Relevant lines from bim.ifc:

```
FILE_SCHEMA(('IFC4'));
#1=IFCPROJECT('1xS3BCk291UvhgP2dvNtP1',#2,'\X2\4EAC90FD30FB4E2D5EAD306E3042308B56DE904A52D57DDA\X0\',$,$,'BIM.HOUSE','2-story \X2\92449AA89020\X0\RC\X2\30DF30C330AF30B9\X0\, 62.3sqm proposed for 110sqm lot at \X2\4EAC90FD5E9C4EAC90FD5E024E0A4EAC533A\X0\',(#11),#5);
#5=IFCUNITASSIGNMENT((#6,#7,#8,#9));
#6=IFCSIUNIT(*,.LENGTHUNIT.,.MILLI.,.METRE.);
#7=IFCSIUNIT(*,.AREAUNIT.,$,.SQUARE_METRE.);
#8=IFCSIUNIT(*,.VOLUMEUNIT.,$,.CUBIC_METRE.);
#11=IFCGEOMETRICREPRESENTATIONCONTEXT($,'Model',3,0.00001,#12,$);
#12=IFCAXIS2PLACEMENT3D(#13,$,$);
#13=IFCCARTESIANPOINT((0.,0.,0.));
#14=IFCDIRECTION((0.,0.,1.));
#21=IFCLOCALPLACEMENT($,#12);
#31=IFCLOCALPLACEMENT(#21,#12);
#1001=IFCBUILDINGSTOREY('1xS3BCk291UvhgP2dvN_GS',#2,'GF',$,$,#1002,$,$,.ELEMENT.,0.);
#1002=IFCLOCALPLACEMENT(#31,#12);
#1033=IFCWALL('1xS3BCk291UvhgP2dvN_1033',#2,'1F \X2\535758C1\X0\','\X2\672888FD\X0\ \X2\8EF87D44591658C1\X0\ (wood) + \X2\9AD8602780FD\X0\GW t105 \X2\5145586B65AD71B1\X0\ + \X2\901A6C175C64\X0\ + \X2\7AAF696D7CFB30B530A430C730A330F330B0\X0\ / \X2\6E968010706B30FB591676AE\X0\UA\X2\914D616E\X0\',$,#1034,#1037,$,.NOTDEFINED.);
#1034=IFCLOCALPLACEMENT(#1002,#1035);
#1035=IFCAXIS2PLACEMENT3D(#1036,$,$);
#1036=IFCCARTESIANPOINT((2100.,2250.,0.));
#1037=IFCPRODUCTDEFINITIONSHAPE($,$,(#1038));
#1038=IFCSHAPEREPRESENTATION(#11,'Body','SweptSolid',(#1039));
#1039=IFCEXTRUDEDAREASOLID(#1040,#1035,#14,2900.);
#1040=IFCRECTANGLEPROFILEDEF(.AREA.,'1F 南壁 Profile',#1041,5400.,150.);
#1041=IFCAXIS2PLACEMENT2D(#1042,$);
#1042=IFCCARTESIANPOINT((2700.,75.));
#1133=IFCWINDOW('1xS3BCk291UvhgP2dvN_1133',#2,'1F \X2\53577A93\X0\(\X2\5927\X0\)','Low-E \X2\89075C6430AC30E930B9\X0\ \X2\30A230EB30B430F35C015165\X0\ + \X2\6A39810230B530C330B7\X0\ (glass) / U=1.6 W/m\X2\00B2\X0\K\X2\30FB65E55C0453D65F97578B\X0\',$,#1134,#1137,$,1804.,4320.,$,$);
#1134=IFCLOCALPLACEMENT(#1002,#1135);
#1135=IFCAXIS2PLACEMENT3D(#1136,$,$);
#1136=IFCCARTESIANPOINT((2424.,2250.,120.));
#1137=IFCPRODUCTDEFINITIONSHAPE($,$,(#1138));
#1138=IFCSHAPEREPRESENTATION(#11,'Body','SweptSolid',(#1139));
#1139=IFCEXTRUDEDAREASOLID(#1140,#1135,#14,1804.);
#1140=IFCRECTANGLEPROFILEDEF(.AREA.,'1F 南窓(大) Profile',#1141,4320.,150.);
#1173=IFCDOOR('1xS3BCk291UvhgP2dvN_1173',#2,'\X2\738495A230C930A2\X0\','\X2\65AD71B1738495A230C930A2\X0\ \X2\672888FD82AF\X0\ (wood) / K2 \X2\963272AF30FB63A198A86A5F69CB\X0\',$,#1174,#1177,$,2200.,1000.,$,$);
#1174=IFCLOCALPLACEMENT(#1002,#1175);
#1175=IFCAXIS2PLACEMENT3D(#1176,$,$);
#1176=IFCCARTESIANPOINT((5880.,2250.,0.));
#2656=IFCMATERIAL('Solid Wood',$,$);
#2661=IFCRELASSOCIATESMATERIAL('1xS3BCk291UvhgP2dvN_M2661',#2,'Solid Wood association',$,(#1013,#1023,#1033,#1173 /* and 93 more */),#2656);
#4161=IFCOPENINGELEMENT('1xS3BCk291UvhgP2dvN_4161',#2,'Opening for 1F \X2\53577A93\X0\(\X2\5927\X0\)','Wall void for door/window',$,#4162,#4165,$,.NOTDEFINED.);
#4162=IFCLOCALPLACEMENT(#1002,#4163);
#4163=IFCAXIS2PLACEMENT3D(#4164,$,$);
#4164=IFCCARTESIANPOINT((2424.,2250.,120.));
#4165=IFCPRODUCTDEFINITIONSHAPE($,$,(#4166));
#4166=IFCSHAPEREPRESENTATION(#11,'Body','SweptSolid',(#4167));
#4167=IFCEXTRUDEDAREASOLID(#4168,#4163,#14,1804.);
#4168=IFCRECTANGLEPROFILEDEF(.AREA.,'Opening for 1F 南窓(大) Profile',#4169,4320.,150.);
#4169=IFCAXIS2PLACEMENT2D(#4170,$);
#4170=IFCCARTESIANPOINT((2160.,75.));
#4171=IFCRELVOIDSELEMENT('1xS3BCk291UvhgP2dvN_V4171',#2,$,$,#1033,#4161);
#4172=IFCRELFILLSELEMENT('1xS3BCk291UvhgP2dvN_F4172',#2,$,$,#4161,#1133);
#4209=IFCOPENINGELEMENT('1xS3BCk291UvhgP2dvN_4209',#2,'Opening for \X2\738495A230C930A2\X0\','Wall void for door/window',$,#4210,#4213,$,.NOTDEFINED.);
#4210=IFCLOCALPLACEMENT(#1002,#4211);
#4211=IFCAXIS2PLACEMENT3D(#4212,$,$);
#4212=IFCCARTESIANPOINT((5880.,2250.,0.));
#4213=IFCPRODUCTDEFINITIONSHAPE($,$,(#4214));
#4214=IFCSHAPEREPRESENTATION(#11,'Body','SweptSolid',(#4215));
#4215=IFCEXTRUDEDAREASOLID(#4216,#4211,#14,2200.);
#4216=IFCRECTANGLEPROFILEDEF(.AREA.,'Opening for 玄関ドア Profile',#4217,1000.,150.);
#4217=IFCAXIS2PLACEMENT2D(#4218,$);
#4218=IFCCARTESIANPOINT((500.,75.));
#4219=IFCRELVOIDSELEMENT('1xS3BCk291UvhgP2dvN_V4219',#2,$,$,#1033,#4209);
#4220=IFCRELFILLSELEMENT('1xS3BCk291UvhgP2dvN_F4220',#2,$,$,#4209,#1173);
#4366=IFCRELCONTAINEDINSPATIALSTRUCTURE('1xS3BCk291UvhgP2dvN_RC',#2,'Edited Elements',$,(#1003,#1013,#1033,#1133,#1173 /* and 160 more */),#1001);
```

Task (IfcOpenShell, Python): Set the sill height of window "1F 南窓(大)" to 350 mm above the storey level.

```python
import numpy as np
import ifcopenshell
import ifcopenshell.api.geometry
import ifcopenshell.geom
import ifcopenshell.util.element
import ifcopenshell.util.placement
import ifcopenshell.util.shape
import ifcopenshell.util.unit

model = ifcopenshell.open("bim.ifc")
unit_scale = ifcopenshell.util.unit.calculate_unit_scale(model)

window = model.by_guid("1xS3BCk291UvhgP2dvN_1133")
opening = window.FillsVoids[0].RelatingOpeningElement
storey = ifcopenshell.util.element.get_container(window, ifc_class="IfcBuildingStorey")
level = ifcopenshell.util.placement.get_local_placement(storey.ObjectPlacement)[2, 3]

# The opening's origin need not be at the sill, so measure its lowest point.
shape = ifcopenshell.geom.create_shape(ifcopenshell.geom.settings(), opening)
bottom = ifcopenshell.util.shape.get_shape_bottom_elevation(shape, shape.geometry) / unit_scale
dz = level + 350.0 - bottom

shift = np.array([0.0, 0.0, dz])
# The window is not placed relative to its opening, so move both.
for product in (opening, window):
    matrix = ifcopenshell.util.placement.get_local_placement(product.ObjectPlacement)
    matrix[:3, 3] += shift
    ifcopenshell.api.geometry.edit_object_placement(model, product=product, matrix=matrix, is_si=False)

print(f"moved by {dz * unit_scale:+.3f} m")

model.write("bim_edited.ifc")
```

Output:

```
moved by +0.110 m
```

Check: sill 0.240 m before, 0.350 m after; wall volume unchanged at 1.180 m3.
